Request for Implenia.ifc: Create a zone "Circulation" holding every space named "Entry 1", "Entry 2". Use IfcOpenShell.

First a look at what the model holds.

```python
import ifcopenshell

model = ifcopenshell.open("Implenia.ifc")
print(model.schema)
seen = {}
for space in model.by_type("IfcSpace"):
    seen[space.LongName] = seen.get(space.LongName, 0) + 1
for name, count in sorted(seen.items(), key=str):
    print(count, "x", name)
print("zones:", [z.Name for z in model.by_type("IfcZone")][:20])
```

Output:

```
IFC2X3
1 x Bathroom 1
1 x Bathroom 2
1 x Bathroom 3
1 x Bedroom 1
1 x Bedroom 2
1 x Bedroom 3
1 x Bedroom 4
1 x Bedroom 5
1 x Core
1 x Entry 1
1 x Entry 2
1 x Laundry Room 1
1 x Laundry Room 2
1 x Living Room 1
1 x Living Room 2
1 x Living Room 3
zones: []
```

```python
import ifcopenshell
import ifcopenshell.api.group
import ifcopenshell.api.root

model = ifcopenshell.open("Implenia.ifc")

names = {"Entry 1", "Entry 2"}
spaces = [s for s in model.by_type("IfcSpace") if s.LongName in names]

zone = ifcopenshell.api.root.create_entity(model, ifc_class="IfcZone", name="Circulation")
ifcopenshell.api.group.assign_group(model, products=spaces, group=zone)
print(len(spaces), "spaces in", zone.Name)

model.write("Implenia-out.ifc")
```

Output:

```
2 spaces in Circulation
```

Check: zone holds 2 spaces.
